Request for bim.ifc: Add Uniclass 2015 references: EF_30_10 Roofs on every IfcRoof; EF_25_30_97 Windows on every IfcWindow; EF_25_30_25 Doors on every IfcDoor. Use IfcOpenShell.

First a look at what the model holds.

```python
import ifcopenshell

model = ifcopenshell.open("bim.ifc")
print(model.schema)
print("classifications:", [c.Name for c in model.by_type("IfcClassification")])
for ifc_class in ("IfcDoor", "IfcRoof", "IfcStair", "IfcWall", "IfcWindow"):
    print(ifc_class, len(model.by_type(ifc_class)))
```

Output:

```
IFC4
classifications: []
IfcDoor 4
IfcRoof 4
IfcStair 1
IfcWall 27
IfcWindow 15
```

```python
import ifcopenshell
import ifcopenshell.api.classification

model = ifcopenshell.open("bim.ifc")

system = ifcopenshell.api.classification.add_classification(model, classification="Uniclass 2015")

codes = {
    "IfcRoof": ("EF_30_10", "Roofs"),
    "IfcWindow": ("EF_25_30_97", "Windows"),
    "IfcDoor": ("EF_25_30_25", "Doors"),
}
for ifc_class, (code, name) in codes.items():
    products = model.by_type(ifc_class)
    ifcopenshell.api.classification.add_reference(
        model, products=products, classification=system, identification=code, name=name
    )
    print(code, len(products))

model.write("bim-out.ifc")
```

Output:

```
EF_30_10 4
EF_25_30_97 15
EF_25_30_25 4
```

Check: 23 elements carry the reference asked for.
